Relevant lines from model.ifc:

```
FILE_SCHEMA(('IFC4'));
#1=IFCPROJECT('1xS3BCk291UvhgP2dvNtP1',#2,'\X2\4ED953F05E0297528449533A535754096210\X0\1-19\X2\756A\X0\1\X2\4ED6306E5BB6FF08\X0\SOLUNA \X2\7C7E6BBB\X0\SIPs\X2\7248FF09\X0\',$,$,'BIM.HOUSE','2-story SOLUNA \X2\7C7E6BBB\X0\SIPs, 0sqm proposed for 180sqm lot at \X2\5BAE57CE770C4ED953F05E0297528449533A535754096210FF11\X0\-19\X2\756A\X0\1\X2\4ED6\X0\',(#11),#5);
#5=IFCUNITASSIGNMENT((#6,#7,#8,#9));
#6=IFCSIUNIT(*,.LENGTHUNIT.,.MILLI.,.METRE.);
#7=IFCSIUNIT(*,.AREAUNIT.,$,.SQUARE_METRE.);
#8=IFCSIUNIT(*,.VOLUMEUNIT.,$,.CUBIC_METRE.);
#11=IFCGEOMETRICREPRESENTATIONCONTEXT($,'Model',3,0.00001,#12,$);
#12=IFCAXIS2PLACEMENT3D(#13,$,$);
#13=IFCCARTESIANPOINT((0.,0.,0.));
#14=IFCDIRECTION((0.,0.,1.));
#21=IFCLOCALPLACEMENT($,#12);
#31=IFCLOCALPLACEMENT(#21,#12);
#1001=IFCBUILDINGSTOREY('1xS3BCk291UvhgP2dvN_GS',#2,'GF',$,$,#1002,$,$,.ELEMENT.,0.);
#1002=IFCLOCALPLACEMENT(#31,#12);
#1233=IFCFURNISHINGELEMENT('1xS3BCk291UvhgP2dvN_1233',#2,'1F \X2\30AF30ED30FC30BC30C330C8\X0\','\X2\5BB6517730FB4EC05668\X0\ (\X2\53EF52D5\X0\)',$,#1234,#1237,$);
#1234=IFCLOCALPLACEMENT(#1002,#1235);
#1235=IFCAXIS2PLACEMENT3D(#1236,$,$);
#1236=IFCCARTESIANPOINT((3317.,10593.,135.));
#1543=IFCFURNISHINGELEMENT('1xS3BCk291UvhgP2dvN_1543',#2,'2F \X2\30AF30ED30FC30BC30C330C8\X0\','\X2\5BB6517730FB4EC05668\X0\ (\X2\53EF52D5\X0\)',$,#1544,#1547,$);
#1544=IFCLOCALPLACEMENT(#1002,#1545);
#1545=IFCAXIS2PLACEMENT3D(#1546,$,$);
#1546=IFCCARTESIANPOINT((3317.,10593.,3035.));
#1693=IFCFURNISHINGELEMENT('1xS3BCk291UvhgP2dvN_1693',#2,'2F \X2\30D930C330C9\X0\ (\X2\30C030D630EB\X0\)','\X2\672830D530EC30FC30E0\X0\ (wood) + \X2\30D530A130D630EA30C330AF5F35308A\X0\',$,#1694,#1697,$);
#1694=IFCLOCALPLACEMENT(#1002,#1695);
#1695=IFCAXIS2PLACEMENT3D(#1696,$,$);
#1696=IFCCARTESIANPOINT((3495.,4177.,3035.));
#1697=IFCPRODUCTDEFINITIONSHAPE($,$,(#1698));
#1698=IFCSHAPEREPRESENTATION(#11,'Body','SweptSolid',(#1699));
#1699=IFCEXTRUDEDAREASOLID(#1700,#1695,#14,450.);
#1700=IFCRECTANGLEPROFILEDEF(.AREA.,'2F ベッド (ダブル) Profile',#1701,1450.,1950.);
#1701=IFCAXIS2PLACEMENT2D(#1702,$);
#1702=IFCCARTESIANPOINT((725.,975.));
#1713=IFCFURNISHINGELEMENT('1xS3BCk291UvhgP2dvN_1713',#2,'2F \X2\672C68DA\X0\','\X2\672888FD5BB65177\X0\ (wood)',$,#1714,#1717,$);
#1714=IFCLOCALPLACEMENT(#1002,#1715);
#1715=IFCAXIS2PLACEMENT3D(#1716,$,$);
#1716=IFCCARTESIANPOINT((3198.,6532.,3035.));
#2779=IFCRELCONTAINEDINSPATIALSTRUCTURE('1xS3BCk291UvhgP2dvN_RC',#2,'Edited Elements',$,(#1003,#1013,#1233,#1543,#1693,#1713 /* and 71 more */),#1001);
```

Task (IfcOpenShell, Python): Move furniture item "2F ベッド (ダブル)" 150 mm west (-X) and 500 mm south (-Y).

```python
import ifcopenshell
import ifcopenshell.api.geometry
import ifcopenshell.util.placement
import ifcopenshell.util.unit

model = ifcopenshell.open("model.ifc")
unit_scale = ifcopenshell.util.unit.calculate_unit_scale(model)

item = model.by_id(1693)
matrix = ifcopenshell.util.placement.get_local_placement(item.ObjectPlacement)
matrix[0, 3] -= 0.15 / unit_scale
matrix[1, 3] -= 0.5 / unit_scale
ifcopenshell.api.geometry.edit_object_placement(model, product=item, matrix=matrix, is_si=False)

print(ifcopenshell.util.placement.get_local_placement(item.ObjectPlacement).round(3) + 0.0)

model.write("model_v2.ifc")
```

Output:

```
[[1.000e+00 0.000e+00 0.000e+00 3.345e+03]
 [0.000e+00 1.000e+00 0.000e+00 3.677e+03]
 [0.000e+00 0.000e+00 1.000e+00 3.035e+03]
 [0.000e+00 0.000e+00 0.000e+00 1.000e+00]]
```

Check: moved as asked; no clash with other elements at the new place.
